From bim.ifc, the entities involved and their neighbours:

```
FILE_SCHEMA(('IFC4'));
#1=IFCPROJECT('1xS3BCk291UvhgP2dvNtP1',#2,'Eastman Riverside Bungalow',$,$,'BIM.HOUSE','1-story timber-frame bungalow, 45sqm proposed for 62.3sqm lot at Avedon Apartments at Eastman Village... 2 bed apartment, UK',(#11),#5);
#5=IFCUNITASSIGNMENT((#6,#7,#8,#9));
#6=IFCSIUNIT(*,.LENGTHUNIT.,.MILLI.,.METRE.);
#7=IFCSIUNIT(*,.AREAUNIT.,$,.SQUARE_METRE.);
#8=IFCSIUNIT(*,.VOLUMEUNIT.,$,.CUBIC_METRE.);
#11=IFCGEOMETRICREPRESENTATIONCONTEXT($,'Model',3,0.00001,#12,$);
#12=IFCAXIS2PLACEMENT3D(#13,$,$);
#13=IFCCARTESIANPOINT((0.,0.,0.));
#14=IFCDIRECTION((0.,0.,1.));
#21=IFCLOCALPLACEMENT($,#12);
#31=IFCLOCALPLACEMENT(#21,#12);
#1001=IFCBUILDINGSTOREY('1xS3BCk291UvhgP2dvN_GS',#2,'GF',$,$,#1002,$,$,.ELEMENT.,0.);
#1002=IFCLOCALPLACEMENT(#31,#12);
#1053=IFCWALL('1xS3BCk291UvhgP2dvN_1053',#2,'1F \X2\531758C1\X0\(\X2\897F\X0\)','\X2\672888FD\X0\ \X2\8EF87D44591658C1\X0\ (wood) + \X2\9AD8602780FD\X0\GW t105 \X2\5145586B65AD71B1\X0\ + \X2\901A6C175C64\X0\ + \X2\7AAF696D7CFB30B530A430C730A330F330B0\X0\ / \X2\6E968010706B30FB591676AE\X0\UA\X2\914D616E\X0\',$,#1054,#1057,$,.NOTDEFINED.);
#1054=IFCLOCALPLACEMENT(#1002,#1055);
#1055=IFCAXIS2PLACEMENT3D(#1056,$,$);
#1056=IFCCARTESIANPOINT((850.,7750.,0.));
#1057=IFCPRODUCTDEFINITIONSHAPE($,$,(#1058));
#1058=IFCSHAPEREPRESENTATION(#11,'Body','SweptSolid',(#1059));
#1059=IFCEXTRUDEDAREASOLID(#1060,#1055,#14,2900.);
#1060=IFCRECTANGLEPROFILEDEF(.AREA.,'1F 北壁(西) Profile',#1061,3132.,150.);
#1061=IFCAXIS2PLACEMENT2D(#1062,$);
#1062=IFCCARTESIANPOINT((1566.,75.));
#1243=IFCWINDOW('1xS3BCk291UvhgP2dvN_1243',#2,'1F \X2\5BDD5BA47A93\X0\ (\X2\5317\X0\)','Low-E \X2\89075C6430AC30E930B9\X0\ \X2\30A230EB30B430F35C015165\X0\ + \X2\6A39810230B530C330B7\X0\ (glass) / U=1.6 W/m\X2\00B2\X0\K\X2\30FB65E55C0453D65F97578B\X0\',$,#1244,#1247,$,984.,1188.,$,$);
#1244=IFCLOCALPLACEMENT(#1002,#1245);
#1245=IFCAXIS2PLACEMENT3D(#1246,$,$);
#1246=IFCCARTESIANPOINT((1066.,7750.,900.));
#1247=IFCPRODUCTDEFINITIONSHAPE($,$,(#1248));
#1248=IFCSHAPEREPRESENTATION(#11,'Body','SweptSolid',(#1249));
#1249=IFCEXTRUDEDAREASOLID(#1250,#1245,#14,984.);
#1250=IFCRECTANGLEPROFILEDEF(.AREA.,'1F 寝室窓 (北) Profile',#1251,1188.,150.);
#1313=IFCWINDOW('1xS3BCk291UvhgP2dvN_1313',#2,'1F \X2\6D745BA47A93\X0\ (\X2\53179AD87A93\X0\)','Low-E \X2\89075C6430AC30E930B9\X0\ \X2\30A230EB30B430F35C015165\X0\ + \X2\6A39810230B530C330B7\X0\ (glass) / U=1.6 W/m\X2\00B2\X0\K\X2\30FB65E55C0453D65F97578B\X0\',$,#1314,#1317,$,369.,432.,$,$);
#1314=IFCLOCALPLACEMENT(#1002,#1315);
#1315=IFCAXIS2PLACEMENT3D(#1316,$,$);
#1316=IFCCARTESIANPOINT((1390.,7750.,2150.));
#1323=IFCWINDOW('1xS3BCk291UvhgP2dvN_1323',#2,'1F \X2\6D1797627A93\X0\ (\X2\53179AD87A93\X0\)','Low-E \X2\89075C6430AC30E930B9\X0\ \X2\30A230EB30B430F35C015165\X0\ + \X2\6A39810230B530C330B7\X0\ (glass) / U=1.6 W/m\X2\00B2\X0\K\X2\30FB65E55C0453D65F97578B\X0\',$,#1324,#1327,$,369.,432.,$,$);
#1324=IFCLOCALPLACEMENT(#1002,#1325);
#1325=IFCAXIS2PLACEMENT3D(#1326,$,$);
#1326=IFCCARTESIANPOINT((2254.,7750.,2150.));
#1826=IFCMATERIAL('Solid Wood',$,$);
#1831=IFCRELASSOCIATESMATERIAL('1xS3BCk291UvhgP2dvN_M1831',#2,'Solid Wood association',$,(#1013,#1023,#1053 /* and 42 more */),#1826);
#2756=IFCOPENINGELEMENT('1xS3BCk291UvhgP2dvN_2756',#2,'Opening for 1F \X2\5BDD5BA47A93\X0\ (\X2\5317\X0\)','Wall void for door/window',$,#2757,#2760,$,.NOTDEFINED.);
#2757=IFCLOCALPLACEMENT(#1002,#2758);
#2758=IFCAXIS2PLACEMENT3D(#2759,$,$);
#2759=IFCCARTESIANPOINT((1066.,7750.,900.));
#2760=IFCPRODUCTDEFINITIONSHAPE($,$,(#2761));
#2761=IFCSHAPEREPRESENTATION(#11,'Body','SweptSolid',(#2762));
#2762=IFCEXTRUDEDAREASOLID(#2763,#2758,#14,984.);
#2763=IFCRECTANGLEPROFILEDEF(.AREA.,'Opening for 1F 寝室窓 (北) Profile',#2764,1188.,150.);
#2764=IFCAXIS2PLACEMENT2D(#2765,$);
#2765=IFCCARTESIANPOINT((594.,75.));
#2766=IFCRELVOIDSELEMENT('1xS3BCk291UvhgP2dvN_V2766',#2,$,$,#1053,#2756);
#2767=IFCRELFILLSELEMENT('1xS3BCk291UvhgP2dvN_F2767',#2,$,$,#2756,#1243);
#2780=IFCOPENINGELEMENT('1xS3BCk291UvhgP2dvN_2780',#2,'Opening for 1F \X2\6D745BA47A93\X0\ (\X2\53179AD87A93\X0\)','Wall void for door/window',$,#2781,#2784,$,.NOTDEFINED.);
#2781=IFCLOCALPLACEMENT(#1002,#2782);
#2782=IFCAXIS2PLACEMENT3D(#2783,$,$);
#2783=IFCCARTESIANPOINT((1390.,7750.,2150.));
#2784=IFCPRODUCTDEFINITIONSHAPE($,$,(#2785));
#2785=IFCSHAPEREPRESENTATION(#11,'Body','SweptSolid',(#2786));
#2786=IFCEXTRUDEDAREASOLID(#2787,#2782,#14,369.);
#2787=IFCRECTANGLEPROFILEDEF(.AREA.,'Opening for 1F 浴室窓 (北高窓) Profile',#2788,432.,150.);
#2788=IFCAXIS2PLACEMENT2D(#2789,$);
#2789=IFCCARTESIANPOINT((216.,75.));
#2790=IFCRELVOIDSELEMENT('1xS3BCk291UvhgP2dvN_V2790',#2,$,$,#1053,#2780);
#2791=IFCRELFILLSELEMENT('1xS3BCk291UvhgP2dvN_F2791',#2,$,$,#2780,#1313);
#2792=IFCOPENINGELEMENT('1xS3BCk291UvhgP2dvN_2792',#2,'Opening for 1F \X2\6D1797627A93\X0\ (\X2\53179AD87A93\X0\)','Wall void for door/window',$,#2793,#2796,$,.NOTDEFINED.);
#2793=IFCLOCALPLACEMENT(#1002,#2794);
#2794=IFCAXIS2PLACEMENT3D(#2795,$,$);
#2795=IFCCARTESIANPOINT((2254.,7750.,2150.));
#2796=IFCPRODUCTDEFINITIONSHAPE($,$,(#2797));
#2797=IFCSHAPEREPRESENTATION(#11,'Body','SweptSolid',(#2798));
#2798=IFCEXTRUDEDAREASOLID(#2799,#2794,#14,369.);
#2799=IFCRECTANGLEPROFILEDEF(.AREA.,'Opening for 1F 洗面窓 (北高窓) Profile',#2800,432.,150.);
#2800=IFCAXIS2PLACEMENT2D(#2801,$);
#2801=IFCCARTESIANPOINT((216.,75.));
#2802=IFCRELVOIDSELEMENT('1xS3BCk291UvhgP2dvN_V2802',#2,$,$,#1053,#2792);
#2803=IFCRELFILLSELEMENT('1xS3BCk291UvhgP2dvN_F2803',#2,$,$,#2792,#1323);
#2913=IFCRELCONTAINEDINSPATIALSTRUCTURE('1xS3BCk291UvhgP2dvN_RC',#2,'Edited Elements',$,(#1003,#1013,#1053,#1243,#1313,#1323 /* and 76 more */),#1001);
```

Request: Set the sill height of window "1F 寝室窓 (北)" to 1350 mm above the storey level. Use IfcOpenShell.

```python
import numpy as np
import ifcopenshell
import ifcopenshell.api.geometry
import ifcopenshell.geom
import ifcopenshell.util.element
import ifcopenshell.util.placement
import ifcopenshell.util.shape
import ifcopenshell.util.unit

model = ifcopenshell.open("bim.ifc")
unit_scale = ifcopenshell.util.unit.calculate_unit_scale(model)

window = model.by_guid("1xS3BCk291UvhgP2dvN_1243")
opening = window.FillsVoids[0].RelatingOpeningElement
storey = ifcopenshell.util.element.get_container(window, ifc_class="IfcBuildingStorey")
level = ifcopenshell.util.placement.get_local_placement(storey.ObjectPlacement)[2, 3]

# The opening's origin need not be at the sill, so measure its lowest point.
shape = ifcopenshell.geom.create_shape(ifcopenshell.geom.settings(), opening)
bottom = ifcopenshell.util.shape.get_shape_bottom_elevation(shape, shape.geometry) / unit_scale
dz = level + 1350.0 - bottom

shift = np.array([0.0, 0.0, dz])
# The window is not placed relative to its opening, so move both.
for product in (opening, window):
    matrix = ifcopenshell.util.placement.get_local_placement(product.ObjectPlacement)
    matrix[:3, 3] += shift
    ifcopenshell.api.geometry.edit_object_placement(model, product=product, matrix=matrix, is_si=False)

print(f"moved by {dz * unit_scale:+.3f} m")

model.write("bim_edited.ifc")
```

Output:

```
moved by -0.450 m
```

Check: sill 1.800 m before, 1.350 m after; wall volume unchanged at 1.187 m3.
